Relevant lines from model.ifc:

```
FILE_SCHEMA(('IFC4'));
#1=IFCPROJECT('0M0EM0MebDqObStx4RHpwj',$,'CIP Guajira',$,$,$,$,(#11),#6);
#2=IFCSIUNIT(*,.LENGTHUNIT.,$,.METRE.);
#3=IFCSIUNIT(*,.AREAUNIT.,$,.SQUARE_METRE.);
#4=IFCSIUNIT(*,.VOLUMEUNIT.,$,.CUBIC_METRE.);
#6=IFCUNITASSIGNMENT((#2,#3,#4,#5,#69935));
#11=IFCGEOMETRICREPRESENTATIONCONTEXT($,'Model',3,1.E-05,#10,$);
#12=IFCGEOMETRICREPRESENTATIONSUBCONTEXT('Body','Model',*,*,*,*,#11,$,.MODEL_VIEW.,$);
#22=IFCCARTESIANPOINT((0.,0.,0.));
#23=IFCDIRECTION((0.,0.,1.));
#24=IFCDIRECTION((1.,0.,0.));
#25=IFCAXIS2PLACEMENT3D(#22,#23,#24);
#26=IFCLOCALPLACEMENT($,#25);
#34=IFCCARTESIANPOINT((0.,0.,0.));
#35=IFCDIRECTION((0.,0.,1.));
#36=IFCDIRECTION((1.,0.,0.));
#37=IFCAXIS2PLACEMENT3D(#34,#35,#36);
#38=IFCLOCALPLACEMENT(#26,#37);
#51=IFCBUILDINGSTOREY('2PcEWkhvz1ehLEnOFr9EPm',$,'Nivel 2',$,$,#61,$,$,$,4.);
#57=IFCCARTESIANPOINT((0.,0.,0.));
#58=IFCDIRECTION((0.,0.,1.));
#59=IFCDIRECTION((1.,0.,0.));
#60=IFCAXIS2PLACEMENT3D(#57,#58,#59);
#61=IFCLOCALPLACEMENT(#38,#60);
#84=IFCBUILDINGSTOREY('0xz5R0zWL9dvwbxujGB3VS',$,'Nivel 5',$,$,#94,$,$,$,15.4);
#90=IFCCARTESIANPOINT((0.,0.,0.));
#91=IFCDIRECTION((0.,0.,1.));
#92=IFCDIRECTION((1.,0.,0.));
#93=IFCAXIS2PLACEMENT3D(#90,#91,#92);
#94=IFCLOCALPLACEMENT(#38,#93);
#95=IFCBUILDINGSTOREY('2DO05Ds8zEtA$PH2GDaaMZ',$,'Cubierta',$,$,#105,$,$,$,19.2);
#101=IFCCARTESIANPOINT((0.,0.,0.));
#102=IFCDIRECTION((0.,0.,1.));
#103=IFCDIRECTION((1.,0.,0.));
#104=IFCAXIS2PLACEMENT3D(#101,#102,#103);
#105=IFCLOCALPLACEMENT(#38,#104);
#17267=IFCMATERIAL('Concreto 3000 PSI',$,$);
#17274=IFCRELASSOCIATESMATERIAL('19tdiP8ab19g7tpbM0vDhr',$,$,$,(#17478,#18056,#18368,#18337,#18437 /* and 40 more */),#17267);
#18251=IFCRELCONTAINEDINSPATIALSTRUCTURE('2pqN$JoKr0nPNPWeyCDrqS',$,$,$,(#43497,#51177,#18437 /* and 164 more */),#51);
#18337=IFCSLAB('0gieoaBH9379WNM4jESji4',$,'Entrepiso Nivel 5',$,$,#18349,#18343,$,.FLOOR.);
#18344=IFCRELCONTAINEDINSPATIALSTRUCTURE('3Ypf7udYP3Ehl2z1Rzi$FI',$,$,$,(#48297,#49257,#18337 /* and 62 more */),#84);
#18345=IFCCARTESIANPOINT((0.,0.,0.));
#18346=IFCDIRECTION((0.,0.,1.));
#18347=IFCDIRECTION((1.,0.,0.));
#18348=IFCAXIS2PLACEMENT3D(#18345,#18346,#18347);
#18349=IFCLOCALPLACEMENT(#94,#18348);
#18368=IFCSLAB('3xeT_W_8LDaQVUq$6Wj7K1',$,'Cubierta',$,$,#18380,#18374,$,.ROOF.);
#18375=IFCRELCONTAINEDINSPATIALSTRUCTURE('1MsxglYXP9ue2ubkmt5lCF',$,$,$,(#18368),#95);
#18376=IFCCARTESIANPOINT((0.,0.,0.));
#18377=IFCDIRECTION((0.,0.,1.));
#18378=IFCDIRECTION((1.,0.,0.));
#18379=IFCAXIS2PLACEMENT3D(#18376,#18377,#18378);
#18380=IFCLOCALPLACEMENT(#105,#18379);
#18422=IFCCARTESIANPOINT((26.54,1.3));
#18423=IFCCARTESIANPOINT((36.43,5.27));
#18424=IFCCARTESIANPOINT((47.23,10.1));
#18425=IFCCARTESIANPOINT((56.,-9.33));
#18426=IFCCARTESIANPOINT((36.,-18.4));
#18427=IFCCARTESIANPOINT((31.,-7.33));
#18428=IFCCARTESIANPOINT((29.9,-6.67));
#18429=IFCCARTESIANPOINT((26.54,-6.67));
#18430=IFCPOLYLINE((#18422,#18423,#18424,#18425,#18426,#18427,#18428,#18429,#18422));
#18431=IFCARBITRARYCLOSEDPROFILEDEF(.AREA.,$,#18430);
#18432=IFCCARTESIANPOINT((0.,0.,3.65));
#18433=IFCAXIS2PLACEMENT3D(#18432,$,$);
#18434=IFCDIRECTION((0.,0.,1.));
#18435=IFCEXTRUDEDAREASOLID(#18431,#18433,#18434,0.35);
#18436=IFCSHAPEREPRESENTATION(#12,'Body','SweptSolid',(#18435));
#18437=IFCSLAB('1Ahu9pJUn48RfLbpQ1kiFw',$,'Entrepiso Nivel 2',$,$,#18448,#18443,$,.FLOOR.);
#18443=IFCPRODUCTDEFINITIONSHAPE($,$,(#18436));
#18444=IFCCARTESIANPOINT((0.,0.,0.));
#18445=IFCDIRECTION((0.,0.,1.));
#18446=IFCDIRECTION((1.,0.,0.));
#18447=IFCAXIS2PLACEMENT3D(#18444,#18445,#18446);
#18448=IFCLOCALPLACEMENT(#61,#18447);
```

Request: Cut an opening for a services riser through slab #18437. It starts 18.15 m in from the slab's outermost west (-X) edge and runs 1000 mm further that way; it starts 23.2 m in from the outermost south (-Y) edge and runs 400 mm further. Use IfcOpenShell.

```python
import numpy as np
import ifcopenshell
import ifcopenshell.api.feature
import ifcopenshell.api.geometry
import ifcopenshell.api.root
import ifcopenshell.geom
import ifcopenshell.util.placement
import ifcopenshell.util.representation
import ifcopenshell.util.shape
import ifcopenshell.util.unit

model = ifcopenshell.open("model.ifc")
unit_scale = ifcopenshell.util.unit.calculate_unit_scale(model)
settings = ifcopenshell.geom.settings()


def volume(element):
    """Net volume in cubic metres, openings subtracted."""
    shape = ifcopenshell.geom.create_shape(settings, element)
    return ifcopenshell.util.shape.get_volume(shape.geometry)


slab = model.by_id(18437)
before = volume(slab)

# Extent in the slab's own axes, in metres. The edges named are its -X and -Y sides.
slab_shape = ifcopenshell.geom.create_shape(settings, slab)
vertices = ifcopenshell.util.shape.get_vertices(slab_shape.geometry)
x_min, y_min, bottom = vertices.min(axis=0)
top = vertices[:, 2].max()

opening = ifcopenshell.api.root.create_entity(model, ifc_class="IfcOpeningElement", name="Services riser opening", predefined_type="OPENING")
context = ifcopenshell.util.representation.get_context(model, "Model", "Body", "MODEL_VIEW")
width, depth = 1, 0.4
outline = [(0.0, 0.0), (width, 0.0), (width, depth), (0.0, depth), (0.0, 0.0)]
# Overshoot both faces by 50 mm so the cut is clean.
shape = ifcopenshell.api.geometry.add_slab_representation(
    model, context=context, depth=top - bottom + 0.1, polyline=outline
)
ifcopenshell.api.geometry.assign_representation(model, product=opening, representation=shape)

matrix = ifcopenshell.util.placement.get_local_placement(slab.ObjectPlacement)
matrix[:, 3] = matrix @ np.append(np.array([x_min + 18.15, y_min + 23.2, bottom - 0.05]) / unit_scale, 1.0)
ifcopenshell.api.geometry.edit_object_placement(model, product=opening, matrix=matrix, is_si=False)
ifcopenshell.api.feature.add_feature(model, feature=opening, element=slab)

after = volume(slab)

print(f"slab volume {before:.3f} -> {after:.3f} m3")

model.write("model-out.ifc")
```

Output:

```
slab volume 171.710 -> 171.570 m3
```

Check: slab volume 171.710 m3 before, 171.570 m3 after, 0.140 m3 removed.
